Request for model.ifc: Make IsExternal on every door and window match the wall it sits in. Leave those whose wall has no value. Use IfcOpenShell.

First a look at what the model holds.

```python
import ifcopenshell
import ifcopenshell.util.element

model = ifcopenshell.open("model.ifc")
print(model.schema)
seen = {}
for e in model.by_type("IfcDoor") + model.by_type("IfcWindow"):
    if not e.FillsVoids:
        continue
    host = e.FillsVoids[0].RelatingOpeningElement.VoidsElements[0].RelatingBuildingElement
    own = ifcopenshell.util.element.get_pset(e, f"Pset_{e.is_a()[3:].removesuffix('StandardCase')}Common", "IsExternal")
    wall = ifcopenshell.util.element.get_pset(host, "Pset_WallCommon", "IsExternal")
    seen[e.is_a(), own, wall] = seen.get((e.is_a(), own, wall), 0) + 1
for (cls, own, wall), count in sorted(seen.items(), key=str):
    print(count, cls, "IsExternal:", own, "| host wall:", wall)
```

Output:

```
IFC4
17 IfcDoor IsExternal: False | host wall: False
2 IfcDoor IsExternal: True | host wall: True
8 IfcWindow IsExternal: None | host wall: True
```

```python
import ifcopenshell
import ifcopenshell.api.pset
import ifcopenshell.util.element

model = ifcopenshell.open("model.ifc")

count = 0
for ifc_class, pset_name in (("IfcDoor", "Pset_DoorCommon"), ("IfcWindow", "Pset_WindowCommon")):
    for e in model.by_type(ifc_class):
        if not e.FillsVoids:
            continue
        host = e.FillsVoids[0].RelatingOpeningElement.VoidsElements[0].RelatingBuildingElement
        external = ifcopenshell.util.element.get_pset(host, "Pset_WallCommon", "IsExternal")
        if external is None or ifcopenshell.util.element.get_pset(e, pset_name, "IsExternal") == external:
            continue
        pset = ifcopenshell.api.pset.add_pset(model, product=e, name=pset_name)
        ifcopenshell.api.pset.edit_pset(model, pset=pset, properties={"IsExternal": external})
        count += 1

print(count, "updated")

model.write("model_updated.ifc")
```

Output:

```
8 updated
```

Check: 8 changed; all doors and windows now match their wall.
